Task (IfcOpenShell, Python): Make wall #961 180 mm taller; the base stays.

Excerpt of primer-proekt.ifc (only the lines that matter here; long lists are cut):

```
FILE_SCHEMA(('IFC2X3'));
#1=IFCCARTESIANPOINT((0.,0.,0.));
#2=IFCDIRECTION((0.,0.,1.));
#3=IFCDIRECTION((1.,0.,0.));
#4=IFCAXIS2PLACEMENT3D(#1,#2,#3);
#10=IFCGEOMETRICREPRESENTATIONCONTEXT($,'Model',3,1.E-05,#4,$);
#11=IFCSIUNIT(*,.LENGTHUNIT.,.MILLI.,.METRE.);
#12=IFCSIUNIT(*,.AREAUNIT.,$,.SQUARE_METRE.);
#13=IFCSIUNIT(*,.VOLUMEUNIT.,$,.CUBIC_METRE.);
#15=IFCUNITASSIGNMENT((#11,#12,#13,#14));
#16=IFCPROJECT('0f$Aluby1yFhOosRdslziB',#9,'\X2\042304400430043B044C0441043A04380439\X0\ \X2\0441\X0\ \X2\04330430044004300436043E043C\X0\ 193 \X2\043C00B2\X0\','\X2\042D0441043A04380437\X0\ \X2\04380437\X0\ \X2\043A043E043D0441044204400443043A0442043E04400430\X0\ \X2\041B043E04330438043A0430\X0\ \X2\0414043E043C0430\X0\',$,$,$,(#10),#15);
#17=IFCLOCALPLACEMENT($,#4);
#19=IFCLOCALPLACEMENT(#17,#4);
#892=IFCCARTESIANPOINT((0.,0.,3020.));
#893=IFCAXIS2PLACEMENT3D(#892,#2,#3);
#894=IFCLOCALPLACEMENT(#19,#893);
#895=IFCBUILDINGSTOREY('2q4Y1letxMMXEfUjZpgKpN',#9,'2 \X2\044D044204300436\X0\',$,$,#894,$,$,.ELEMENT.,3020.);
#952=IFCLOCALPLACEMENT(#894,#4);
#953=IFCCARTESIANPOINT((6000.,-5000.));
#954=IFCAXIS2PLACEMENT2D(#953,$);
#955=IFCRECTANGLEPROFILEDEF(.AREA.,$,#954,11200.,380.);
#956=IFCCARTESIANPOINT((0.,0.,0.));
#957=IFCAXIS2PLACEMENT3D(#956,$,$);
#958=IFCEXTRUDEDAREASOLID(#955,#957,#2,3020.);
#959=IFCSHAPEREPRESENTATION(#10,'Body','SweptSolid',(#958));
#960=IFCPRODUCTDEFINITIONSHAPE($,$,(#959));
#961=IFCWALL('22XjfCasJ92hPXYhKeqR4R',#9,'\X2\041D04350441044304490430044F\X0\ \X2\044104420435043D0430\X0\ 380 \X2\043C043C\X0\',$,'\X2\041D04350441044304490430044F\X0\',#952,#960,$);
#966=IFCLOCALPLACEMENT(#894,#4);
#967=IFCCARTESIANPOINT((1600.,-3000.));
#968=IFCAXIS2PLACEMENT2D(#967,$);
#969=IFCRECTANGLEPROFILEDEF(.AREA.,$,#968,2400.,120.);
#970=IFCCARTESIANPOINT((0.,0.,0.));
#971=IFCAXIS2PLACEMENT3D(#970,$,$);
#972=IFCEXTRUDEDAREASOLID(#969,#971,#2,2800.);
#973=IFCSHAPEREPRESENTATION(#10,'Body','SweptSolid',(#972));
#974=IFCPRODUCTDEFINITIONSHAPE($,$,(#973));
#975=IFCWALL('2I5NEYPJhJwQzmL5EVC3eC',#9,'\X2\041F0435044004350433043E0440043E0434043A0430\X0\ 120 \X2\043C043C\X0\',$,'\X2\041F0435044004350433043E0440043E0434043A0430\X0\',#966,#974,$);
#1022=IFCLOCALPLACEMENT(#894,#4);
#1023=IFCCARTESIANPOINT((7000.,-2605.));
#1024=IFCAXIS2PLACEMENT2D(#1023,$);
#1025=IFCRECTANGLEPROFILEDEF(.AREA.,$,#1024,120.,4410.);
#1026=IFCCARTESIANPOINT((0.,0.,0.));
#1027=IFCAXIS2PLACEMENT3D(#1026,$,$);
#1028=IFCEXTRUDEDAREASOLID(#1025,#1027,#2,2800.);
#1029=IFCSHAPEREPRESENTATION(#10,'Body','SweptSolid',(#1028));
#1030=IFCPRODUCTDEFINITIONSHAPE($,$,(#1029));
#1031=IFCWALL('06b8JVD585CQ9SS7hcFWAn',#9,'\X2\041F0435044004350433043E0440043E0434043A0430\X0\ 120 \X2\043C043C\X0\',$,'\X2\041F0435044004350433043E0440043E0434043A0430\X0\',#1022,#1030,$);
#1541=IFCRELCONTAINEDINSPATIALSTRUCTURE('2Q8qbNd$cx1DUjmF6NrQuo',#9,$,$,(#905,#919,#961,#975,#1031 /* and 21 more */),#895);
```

```python
import ifcopenshell
import ifcopenshell.geom
import ifcopenshell.util.shape
import ifcopenshell.util.unit

model = ifcopenshell.open("primer-proekt.ifc")
unit_scale = ifcopenshell.util.unit.calculate_unit_scale(model)
settings = ifcopenshell.geom.settings()


def volume(element):
    """Net volume in cubic metres, openings subtracted."""
    shape = ifcopenshell.geom.create_shape(settings, element)
    return ifcopenshell.util.shape.get_volume(shape.geometry)


wall = model.by_id(961)
before = volume(wall)

body = next(r for r in wall.Representation.Representations if r.RepresentationIdentifier == "Body")
solid = body.Items[0]
old_height = solid.Depth
solid.Depth += 0.18 / unit_scale
after = volume(wall)

print(f"height {old_height:g} -> {solid.Depth:g}, volume {before:.3f} -> {after:.3f} m3")

model.write("primer-proekt_updated.ifc")
```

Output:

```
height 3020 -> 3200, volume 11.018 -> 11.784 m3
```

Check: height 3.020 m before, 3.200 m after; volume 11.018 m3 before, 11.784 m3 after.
